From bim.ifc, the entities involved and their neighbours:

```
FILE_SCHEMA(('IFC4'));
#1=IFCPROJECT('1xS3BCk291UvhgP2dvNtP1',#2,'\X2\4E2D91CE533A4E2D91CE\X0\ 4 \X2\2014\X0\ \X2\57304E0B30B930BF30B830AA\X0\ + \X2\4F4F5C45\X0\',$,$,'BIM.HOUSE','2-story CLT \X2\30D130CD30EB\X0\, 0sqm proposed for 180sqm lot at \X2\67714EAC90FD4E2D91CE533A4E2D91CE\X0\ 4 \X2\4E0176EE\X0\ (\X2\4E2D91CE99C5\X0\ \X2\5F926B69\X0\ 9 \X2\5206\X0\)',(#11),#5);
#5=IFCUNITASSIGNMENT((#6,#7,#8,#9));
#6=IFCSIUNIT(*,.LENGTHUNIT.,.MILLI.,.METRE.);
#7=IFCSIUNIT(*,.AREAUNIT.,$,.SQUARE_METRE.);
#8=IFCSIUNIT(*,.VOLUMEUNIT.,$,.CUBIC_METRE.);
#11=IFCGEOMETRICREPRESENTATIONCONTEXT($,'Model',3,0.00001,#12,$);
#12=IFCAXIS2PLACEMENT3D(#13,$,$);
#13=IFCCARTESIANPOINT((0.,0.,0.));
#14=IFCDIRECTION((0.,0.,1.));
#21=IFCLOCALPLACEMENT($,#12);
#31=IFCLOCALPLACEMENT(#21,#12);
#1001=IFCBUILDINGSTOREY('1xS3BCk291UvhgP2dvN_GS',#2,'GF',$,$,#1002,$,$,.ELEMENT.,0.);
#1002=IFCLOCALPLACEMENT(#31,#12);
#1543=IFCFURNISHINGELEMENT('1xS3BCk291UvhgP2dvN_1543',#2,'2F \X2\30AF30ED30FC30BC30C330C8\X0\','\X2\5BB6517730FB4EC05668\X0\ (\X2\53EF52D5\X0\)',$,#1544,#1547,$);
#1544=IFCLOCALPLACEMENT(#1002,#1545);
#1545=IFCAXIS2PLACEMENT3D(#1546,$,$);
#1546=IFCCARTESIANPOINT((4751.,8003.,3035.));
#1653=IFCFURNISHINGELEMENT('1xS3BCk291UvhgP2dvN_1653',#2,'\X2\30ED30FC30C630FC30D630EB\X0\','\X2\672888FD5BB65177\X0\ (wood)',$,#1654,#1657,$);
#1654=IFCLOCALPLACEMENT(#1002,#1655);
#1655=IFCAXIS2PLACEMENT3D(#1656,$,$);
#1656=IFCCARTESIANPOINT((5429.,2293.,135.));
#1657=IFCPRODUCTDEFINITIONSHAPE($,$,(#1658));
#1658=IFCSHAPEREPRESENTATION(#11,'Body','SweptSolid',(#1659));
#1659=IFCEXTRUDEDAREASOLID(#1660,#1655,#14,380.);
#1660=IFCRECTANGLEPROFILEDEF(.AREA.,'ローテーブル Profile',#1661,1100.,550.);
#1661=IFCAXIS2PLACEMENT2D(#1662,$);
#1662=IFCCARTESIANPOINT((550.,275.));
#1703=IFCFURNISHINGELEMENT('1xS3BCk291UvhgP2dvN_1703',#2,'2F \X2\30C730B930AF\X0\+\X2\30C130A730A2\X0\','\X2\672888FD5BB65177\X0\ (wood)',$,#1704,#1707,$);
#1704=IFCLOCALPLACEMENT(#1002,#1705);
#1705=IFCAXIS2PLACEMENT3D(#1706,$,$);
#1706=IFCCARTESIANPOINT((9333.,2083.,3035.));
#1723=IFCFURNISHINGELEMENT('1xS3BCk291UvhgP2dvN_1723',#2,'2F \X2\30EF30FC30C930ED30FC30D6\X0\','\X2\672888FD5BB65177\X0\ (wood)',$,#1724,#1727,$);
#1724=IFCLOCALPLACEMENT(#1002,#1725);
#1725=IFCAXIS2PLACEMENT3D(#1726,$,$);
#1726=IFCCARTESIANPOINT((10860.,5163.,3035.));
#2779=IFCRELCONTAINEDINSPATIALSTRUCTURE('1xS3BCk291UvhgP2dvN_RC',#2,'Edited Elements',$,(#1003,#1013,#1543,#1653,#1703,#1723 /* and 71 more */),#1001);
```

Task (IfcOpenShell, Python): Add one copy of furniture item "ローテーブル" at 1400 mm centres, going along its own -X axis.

```python
import ifcopenshell
import ifcopenshell.api.geometry
import ifcopenshell.api.root
import ifcopenshell.util.element
import ifcopenshell.util.placement
import ifcopenshell.util.unit

model = ifcopenshell.open("bim.ifc")
unit_scale = ifcopenshell.util.unit.calculate_unit_scale(model)


def reuse_history(source, copy):
    """copy_class also copies each property set's owner history, people and application; keep the originals."""
    for rel in copy.IsDefinedBy:
        if rel.is_a("IfcRelDefinesByProperties") and (history := rel.RelatingPropertyDefinition.OwnerHistory):
            rel.RelatingPropertyDefinition.OwnerHistory = source.OwnerHistory
            ifcopenshell.util.element.remove_deep2(model, history)


source = model.by_guid("1xS3BCk291UvhgP2dvN_1653")
base = ifcopenshell.util.placement.get_local_placement(source.ObjectPlacement)
step = -base[:3, 0] * 1.4 / unit_scale

for i in range(1, 2):
    copy = ifcopenshell.api.root.copy_class(model, product=source)
    copy.Representation = ifcopenshell.util.element.copy_deep(
        model, source.Representation, exclude=["IfcGeometricRepresentationContext", "IfcRepresentationMap"]
    )
    reuse_history(source, copy)
    matrix = base.copy()
    matrix[:3, 3] += i * step
    print("added at", matrix[:3, 3].round(3) + 0.0)
    ifcopenshell.api.geometry.edit_object_placement(model, product=copy, matrix=matrix, is_si=False)

model.write("bim-out.ifc")
```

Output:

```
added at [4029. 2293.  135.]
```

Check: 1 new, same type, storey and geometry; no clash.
